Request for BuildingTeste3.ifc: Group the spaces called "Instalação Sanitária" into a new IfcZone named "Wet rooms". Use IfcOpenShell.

First a look at what the model holds.

```python
import ifcopenshell

model = ifcopenshell.open("BuildingTeste3.ifc")
print(model.schema)
seen = {}
for space in model.by_type("IfcSpace"):
    seen[space.LongName] = seen.get(space.LongName, 0) + 1
for name, count in sorted(seen.items(), key=str):
    print(count, "x", name)
print("zones:", [z.Name for z in model.by_type("IfcZone")][:20])
```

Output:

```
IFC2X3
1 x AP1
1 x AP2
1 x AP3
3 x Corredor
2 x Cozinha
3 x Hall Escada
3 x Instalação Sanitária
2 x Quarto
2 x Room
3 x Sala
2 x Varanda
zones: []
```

```python
import ifcopenshell
import ifcopenshell.api.group
import ifcopenshell.api.root

model = ifcopenshell.open("BuildingTeste3.ifc")

names = {"Instalação Sanitária"}
spaces = [s for s in model.by_type("IfcSpace") if s.LongName in names]

zone = ifcopenshell.api.root.create_entity(model, ifc_class="IfcZone", name="Wet rooms")
ifcopenshell.api.group.assign_group(model, products=spaces, group=zone)
print(len(spaces), "spaces in", zone.Name)

model.write("BuildingTeste3_edited.ifc")
```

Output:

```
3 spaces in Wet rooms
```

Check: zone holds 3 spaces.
